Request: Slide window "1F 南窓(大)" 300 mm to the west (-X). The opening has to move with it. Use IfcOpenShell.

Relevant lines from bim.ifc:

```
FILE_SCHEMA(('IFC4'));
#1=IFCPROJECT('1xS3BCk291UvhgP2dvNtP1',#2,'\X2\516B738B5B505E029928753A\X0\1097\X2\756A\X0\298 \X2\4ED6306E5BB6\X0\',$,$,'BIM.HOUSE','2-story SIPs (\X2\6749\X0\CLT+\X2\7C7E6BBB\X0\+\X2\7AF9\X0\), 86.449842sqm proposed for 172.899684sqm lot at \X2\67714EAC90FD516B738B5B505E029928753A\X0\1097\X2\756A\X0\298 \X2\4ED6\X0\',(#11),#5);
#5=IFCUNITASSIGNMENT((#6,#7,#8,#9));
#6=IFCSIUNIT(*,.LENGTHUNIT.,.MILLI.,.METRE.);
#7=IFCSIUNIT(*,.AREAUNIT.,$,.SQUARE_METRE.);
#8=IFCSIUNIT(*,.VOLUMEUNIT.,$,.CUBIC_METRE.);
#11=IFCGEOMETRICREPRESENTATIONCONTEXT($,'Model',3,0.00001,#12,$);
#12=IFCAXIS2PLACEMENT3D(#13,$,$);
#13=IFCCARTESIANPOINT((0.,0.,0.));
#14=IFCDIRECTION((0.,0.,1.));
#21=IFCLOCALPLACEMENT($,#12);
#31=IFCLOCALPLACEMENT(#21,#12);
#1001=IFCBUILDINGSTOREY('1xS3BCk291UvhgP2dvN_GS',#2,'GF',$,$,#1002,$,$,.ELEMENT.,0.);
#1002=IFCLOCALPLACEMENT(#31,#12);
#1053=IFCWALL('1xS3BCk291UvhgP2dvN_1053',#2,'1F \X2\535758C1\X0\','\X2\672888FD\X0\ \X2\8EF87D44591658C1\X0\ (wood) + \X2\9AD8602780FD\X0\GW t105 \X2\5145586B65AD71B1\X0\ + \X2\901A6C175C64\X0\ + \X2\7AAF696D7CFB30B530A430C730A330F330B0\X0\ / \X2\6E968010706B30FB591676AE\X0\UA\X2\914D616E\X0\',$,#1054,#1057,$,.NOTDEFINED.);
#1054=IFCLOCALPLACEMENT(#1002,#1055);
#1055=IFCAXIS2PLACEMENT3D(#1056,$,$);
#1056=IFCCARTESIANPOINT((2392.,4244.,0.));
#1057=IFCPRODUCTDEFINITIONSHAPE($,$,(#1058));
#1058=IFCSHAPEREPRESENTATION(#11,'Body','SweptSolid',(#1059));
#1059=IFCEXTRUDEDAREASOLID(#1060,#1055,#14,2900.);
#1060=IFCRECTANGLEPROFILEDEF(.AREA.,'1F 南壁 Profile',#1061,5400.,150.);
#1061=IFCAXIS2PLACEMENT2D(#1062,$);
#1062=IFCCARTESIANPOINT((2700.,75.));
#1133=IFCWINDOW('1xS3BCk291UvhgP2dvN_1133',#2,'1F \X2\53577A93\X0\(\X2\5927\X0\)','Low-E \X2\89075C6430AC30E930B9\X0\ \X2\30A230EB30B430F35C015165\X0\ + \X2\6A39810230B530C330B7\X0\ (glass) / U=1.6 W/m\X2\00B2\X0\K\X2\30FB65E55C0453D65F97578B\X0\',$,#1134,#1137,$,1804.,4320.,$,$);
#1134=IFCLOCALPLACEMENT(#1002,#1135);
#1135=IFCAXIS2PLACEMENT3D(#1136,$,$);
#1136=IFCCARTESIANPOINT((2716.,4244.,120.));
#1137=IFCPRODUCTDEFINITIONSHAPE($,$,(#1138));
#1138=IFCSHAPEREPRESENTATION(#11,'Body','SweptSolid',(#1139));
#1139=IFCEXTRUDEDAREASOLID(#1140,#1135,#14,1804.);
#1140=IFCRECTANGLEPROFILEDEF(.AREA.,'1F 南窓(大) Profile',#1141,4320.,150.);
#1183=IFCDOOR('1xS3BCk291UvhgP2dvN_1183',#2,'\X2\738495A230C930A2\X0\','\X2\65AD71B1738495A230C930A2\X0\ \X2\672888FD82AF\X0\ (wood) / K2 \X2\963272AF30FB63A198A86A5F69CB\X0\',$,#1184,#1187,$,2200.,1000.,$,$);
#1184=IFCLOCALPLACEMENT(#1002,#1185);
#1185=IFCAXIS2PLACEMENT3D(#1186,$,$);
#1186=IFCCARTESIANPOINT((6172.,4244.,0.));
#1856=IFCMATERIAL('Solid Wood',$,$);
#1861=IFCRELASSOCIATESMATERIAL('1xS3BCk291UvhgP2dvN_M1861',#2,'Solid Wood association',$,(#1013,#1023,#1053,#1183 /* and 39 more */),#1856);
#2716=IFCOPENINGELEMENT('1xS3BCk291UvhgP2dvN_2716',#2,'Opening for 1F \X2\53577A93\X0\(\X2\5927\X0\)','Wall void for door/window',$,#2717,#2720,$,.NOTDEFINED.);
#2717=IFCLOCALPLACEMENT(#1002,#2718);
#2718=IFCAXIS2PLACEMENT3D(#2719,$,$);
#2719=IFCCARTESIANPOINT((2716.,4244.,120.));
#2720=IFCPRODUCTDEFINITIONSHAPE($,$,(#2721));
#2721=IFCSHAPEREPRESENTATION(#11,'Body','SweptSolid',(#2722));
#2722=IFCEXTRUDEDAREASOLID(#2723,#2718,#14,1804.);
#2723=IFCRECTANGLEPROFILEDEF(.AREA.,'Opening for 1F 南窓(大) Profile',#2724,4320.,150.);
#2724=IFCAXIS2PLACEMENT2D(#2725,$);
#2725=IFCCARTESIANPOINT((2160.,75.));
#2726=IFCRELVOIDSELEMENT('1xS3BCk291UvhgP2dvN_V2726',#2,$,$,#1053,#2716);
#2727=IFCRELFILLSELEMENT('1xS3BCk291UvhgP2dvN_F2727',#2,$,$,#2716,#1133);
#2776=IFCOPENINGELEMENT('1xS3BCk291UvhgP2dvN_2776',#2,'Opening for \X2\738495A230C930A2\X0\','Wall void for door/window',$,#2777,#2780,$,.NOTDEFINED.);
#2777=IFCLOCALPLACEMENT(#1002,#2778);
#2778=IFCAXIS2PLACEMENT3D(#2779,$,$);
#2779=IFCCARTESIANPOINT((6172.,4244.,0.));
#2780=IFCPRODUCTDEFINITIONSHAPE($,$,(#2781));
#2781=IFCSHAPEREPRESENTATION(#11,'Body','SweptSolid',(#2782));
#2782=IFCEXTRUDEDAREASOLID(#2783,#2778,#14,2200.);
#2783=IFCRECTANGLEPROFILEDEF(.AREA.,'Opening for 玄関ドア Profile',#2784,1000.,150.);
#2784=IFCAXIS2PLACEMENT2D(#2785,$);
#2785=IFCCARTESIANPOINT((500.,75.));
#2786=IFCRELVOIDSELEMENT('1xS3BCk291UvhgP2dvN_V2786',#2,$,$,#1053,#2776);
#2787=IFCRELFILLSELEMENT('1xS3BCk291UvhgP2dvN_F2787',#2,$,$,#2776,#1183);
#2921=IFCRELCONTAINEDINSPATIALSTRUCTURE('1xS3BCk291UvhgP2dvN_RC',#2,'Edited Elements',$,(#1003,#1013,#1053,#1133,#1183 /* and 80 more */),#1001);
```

```python
import ifcopenshell
import ifcopenshell.api.geometry
import ifcopenshell.util.placement

model = ifcopenshell.open("bim.ifc")

window = model.by_guid("1xS3BCk291UvhgP2dvN_1133")
opening = window.FillsVoids[0].RelatingOpeningElement
wall = opening.VoidsElements[0].RelatingBuildingElement

wall_matrix = ifcopenshell.util.placement.get_local_placement(wall.ObjectPlacement)
shift = wall_matrix[:3, 0] * -300.0
before = ifcopenshell.util.placement.get_local_placement(window.ObjectPlacement)[:3, 3].copy()

# The window is not placed relative to its opening, so move both.
for product in (opening, window):
    matrix = ifcopenshell.util.placement.get_local_placement(product.ObjectPlacement)
    matrix[:3, 3] += shift
    ifcopenshell.api.geometry.edit_object_placement(model, product=product, matrix=matrix, is_si=False)

after = ifcopenshell.util.placement.get_local_placement(window.ObjectPlacement)[:3, 3]
print("window moved by", (after - before).round(3) + 0.0)

model.write("bim_updated.ifc")
```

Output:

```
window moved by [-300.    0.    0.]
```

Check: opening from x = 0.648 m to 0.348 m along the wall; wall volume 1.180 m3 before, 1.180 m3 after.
